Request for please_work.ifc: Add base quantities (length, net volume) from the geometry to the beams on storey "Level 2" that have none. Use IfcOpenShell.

First a look at what the model holds.

```python
import ifcopenshell
import ifcopenshell.util.element
import ifcopenshell.util.unit

model = ifcopenshell.open("please_work.ifc")
print(model.schema)
for unit_type in ("LENGTHUNIT", "AREAUNIT", "VOLUMEUNIT"):
    print(unit_type, ifcopenshell.util.unit.calculate_unit_scale(model, unit_type))
storey = next(s for s in model.by_type("IfcBuildingStorey") if s.Name == "Level 2")
beams = [e for e in ifcopenshell.util.element.get_decomposition(storey) if e.is_a("IfcBeam")]
for e in sorted(beams, key=lambda e: e.id()):
    print(e.id(), e.is_a(), e.Name, list(ifcopenshell.util.element.get_psets(e, qtos_only=True)), sep=" | ")
```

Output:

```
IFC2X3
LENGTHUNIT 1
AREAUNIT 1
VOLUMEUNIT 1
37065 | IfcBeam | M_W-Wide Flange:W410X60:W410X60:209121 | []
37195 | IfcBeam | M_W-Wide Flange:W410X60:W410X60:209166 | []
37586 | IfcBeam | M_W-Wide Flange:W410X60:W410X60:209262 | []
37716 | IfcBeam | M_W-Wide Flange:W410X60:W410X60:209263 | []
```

```python
import ifcopenshell
import ifcopenshell.api.pset
import ifcopenshell.geom
import ifcopenshell.util.element
import ifcopenshell.util.shape
import ifcopenshell.util.unit

model = ifcopenshell.open("please_work.ifc")
unit_scale = ifcopenshell.util.unit.calculate_unit_scale(model)
volume_scale = ifcopenshell.util.unit.calculate_unit_scale(model, "VOLUMEUNIT")
settings = ifcopenshell.geom.settings()

storey = next(s for s in model.by_type("IfcBuildingStorey") if s.Name == "Level 2")
beams = [e for e in ifcopenshell.util.element.get_decomposition(storey) if e.is_a("IfcBeam")]

for e in sorted(beams, key=lambda e: e.id()):
    if ifcopenshell.util.element.get_psets(e, qtos_only=True, should_inherit=False):
        continue
    # Geometry comes back in metres, in the element's own axes.
    shape = ifcopenshell.geom.create_shape(settings, e)
    values = {
        "Length": ifcopenshell.util.shape.get_max_xyz(shape.geometry) / unit_scale,
        "NetVolume": ifcopenshell.util.shape.get_volume(shape.geometry) / volume_scale,
    }
    qto = ifcopenshell.api.pset.add_qto(model, product=e, name="BaseQuantities")
    ifcopenshell.api.pset.edit_qto(model, qto=qto, properties=values)
    print(e.id(), {k: round(v, 3) for k, v in values.items()})

model.write("please_work_edited.ifc")
```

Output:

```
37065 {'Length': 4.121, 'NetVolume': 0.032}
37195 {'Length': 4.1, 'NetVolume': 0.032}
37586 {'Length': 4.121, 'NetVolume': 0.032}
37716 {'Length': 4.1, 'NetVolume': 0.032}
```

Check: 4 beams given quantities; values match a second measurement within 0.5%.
